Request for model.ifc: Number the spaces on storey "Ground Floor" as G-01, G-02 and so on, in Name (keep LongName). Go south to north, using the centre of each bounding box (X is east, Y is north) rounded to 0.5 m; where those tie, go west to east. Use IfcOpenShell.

First a look at what the model holds.

```python
import ifcopenshell
import ifcopenshell.util.element
import ifcopenshell.util.placement

model = ifcopenshell.open("model.ifc")
print(model.schema)
storey = next(s for s in model.by_type("IfcBuildingStorey") if s.Name == "Ground Floor")
spaces = [e for e in ifcopenshell.util.element.get_decomposition(storey) if e.is_a("IfcSpace")]
for e in sorted(spaces, key=lambda e: e.id()):
    origin = ifcopenshell.util.placement.get_local_placement(e.ObjectPlacement)[:3, 3]
    print(e.id(), e.Name, e.LongName, origin.round(2) + 0.0, sep=" | ")
```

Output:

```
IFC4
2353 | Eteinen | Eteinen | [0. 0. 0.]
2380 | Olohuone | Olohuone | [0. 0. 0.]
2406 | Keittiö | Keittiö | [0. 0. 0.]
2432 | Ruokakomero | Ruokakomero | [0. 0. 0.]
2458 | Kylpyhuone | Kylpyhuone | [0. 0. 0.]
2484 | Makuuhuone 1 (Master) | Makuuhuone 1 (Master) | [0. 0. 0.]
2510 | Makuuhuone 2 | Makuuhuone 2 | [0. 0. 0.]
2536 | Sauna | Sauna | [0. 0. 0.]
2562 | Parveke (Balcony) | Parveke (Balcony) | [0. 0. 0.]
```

```python
import ifcopenshell
import ifcopenshell.geom
import ifcopenshell.util.element
import ifcopenshell.util.shape

model = ifcopenshell.open("model.ifc")
settings = ifcopenshell.geom.settings()
settings.set("use-world-coords", True)


def centre(element):
    shape = ifcopenshell.geom.create_shape(settings, element)
    return ifcopenshell.util.shape.get_bbox_centroid(shape.geometry)


storey = next(s for s in model.by_type("IfcBuildingStorey") if s.Name == "Ground Floor")
spaces = [e for e in ifcopenshell.util.element.get_decomposition(storey) if e.is_a("IfcSpace")]

# Insertion points can sit at a corner or the storey origin, so sort by the geometry (in metres).
centres = {e: centre(e) for e in spaces}
spaces.sort(key=lambda e: (round(centres[e][1] / 0.5), centres[e][0]))

for i, e in enumerate(spaces, start=1):
    number = f"G-{i:02d}"
    e.Name = number
    print(e.id(), number)

model.write("model_updated.ifc")
```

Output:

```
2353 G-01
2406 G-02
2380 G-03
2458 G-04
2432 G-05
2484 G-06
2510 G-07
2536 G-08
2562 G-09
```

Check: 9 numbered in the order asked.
